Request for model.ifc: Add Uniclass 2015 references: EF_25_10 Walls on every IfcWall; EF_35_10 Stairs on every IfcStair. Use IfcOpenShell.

First a look at what the model holds.

```python
import ifcopenshell

model = ifcopenshell.open("model.ifc")
print(model.schema)
print("classifications:", [c.Name for c in model.by_type("IfcClassification")])
for ifc_class in ("IfcDoor", "IfcRoof", "IfcStair", "IfcWall", "IfcWindow"):
    print(ifc_class, len(model.by_type(ifc_class)))
```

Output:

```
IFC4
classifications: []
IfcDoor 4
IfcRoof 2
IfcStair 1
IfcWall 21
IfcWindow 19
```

```python
import ifcopenshell
import ifcopenshell.api.classification

model = ifcopenshell.open("model.ifc")

system = ifcopenshell.api.classification.add_classification(model, classification="Uniclass 2015")

codes = {
    "IfcWall": ("EF_25_10", "Walls"),
    "IfcStair": ("EF_35_10", "Stairs"),
}
for ifc_class, (code, name) in codes.items():
    products = model.by_type(ifc_class)
    ifcopenshell.api.classification.add_reference(
        model, products=products, classification=system, identification=code, name=name
    )
    print(code, len(products))

model.write("model_edited.ifc")
```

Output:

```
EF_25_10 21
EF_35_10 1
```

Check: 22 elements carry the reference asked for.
